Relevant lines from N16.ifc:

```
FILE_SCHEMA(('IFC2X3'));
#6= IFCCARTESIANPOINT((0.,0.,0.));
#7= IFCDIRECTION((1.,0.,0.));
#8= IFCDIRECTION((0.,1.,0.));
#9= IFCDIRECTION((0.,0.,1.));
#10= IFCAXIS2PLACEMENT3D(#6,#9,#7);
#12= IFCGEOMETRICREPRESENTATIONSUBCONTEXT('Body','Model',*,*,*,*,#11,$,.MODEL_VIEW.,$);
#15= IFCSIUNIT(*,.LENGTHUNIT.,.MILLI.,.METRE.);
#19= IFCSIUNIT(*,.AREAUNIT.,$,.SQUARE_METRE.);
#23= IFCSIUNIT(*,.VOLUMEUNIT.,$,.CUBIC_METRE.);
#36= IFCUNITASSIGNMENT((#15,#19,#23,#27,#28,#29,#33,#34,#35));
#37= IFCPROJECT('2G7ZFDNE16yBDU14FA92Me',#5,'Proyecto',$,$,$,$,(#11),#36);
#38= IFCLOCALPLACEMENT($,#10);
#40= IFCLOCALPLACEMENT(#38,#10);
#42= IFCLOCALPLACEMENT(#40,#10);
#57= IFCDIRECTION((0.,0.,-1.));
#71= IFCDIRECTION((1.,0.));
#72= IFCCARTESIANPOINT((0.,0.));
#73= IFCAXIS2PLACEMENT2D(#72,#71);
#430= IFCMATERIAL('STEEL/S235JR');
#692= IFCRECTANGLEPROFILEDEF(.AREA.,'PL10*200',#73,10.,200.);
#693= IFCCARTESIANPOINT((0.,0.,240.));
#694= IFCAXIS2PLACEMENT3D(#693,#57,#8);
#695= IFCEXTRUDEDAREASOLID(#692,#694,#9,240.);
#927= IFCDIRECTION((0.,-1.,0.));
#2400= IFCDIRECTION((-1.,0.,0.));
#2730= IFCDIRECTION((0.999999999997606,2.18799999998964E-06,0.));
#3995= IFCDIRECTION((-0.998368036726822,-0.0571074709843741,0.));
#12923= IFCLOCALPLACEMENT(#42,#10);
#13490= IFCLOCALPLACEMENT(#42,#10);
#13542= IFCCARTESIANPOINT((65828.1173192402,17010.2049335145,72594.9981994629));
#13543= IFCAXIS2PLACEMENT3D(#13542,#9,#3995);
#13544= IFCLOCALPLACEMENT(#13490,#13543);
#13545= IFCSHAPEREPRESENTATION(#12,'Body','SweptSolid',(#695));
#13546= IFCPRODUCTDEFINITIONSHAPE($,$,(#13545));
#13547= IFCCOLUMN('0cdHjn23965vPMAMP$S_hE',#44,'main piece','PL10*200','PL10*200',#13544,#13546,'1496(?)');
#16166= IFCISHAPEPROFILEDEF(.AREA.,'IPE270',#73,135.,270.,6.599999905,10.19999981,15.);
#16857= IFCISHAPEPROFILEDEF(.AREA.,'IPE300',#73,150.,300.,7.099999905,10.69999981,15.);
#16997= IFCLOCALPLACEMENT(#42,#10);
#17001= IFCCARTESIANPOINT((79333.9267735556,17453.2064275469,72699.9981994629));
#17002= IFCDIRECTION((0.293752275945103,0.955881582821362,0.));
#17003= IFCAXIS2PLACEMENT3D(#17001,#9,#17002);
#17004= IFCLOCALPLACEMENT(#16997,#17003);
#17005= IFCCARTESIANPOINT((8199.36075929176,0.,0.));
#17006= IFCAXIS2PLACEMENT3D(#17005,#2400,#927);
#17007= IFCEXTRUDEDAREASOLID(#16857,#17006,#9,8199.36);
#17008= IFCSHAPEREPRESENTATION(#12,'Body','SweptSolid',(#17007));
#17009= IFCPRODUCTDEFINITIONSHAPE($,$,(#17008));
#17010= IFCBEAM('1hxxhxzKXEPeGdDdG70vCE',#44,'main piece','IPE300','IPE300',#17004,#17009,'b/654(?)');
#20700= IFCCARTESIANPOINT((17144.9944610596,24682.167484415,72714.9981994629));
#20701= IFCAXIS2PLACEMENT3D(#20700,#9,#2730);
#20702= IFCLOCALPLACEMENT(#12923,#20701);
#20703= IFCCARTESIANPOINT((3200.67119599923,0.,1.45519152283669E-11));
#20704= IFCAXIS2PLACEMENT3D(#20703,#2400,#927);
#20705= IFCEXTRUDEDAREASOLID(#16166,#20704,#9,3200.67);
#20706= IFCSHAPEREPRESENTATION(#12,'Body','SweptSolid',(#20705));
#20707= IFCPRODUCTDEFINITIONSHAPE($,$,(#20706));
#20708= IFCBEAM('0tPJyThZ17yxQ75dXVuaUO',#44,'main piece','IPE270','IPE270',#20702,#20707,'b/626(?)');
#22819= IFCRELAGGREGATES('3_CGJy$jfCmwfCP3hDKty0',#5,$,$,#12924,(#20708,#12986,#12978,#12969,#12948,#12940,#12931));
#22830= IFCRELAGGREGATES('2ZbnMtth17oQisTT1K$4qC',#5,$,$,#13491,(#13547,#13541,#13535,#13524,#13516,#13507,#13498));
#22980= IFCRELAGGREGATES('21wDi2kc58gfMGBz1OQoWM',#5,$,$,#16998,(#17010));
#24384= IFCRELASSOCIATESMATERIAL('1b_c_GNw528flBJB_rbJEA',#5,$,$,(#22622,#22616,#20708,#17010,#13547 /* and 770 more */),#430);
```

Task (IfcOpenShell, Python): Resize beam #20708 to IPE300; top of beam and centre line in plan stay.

```python
import ifcopenshell
import ifcopenshell.util.element
import ifcopenshell.util.representation

model = ifcopenshell.open("N16.ifc")

member = model.by_guid("0tPJyThZ17yxQ75dXVuaUO")
source = next(p for p in model.by_type("IfcIShapeProfileDef") if p.ProfileName == "IPE300")

body = ifcopenshell.util.representation.get_representation(member, "Model", "Body")
solid = body.Items[0]
old_profile = solid.SweptArea

# Copy the section's sizes but keep this member's own profile position.
profile = ifcopenshell.util.element.copy(model, source)
# Profiles are centred, so shift by half the change in depth to hold the top.
shift = (old_profile.OverallDepth - profile.OverallDepth) / 2
x, y = old_profile.Position.Location.Coordinates
up = (0.0, 1.0)  # upwards, in the solid's own plane
location = model.createIfcCartesianPoint((x + up[0] * shift, y + up[1] * shift))
profile.Position = model.createIfcAxis2Placement2D(location, old_profile.Position.RefDirection)
solid.SweptArea = profile
if not model.get_total_inverses(old_profile):
    ifcopenshell.util.element.remove_deep2(model, old_profile)
member.Description = member.Description.replace("IPE270", "IPE300")
member.ObjectType = member.ObjectType.replace("IPE270", "IPE300")

print(solid.SweptArea)

model.write("N16_v2.ifc")
```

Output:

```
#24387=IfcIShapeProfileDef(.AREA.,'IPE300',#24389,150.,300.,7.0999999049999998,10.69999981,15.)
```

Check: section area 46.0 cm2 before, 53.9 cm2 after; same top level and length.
